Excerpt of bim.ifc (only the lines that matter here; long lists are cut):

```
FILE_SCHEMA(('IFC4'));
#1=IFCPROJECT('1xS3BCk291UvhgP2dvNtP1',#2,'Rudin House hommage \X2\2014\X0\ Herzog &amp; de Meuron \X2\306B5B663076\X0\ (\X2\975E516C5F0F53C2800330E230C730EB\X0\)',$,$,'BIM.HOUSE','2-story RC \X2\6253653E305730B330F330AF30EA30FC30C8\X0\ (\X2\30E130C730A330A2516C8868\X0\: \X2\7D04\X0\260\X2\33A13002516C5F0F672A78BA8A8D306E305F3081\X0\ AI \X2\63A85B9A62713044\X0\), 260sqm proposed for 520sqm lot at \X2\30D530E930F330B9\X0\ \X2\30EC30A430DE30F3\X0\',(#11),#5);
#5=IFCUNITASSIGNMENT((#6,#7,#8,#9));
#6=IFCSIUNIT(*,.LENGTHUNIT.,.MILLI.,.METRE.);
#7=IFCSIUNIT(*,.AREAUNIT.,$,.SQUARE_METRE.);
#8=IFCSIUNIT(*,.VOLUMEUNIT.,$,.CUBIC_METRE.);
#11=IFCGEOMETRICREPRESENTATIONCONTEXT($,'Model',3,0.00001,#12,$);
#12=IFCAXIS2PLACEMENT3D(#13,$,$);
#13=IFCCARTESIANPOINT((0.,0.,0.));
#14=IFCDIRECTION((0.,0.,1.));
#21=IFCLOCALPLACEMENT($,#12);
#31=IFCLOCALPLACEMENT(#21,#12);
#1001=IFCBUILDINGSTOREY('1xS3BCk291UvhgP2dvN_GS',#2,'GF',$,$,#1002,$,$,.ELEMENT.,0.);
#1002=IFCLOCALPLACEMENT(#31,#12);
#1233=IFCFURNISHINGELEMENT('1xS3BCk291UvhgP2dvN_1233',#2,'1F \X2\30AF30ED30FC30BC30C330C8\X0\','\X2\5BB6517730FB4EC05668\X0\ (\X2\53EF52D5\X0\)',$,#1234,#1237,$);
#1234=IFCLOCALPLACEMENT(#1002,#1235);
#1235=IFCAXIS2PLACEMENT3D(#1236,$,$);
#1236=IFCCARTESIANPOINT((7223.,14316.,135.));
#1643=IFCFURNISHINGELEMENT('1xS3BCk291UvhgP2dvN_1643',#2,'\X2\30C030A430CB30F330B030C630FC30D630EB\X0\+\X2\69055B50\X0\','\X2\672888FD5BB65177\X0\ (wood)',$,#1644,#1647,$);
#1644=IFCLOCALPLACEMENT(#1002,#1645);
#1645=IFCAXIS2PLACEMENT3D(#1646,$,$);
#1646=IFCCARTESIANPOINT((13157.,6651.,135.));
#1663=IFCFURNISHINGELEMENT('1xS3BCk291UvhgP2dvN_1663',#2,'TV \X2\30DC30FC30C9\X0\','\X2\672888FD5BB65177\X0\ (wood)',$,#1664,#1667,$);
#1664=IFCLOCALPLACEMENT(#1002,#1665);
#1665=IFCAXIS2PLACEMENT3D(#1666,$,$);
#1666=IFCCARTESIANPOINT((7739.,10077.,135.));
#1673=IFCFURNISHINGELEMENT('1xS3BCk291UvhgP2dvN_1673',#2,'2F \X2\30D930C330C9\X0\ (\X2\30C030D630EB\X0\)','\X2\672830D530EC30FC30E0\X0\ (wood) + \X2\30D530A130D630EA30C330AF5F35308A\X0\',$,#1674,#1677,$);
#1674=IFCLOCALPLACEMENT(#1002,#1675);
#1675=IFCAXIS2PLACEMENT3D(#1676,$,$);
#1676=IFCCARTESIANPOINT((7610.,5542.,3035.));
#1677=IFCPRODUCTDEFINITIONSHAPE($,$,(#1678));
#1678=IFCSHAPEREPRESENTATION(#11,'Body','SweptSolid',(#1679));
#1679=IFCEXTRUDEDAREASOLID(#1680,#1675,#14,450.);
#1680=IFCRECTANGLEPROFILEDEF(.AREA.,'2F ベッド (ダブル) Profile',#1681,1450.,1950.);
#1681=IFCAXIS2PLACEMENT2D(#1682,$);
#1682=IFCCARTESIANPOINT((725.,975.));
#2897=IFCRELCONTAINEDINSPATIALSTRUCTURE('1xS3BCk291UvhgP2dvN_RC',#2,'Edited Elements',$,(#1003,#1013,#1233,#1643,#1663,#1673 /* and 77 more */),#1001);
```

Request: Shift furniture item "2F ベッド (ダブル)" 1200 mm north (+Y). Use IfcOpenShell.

```python
import ifcopenshell
import ifcopenshell.api.geometry
import ifcopenshell.util.placement
import ifcopenshell.util.unit

model = ifcopenshell.open("bim.ifc")
unit_scale = ifcopenshell.util.unit.calculate_unit_scale(model)

item = model.by_guid("1xS3BCk291UvhgP2dvN_1673")
matrix = ifcopenshell.util.placement.get_local_placement(item.ObjectPlacement)
matrix[1, 3] += 1.2 / unit_scale
ifcopenshell.api.geometry.edit_object_placement(model, product=item, matrix=matrix, is_si=False)

print(ifcopenshell.util.placement.get_local_placement(item.ObjectPlacement).round(3) + 0.0)

model.write("bim_v2.ifc")
```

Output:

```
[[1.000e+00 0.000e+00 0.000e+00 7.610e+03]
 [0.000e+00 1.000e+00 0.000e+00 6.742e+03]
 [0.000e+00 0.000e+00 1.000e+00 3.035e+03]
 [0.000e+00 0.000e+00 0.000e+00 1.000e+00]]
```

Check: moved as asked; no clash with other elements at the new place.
